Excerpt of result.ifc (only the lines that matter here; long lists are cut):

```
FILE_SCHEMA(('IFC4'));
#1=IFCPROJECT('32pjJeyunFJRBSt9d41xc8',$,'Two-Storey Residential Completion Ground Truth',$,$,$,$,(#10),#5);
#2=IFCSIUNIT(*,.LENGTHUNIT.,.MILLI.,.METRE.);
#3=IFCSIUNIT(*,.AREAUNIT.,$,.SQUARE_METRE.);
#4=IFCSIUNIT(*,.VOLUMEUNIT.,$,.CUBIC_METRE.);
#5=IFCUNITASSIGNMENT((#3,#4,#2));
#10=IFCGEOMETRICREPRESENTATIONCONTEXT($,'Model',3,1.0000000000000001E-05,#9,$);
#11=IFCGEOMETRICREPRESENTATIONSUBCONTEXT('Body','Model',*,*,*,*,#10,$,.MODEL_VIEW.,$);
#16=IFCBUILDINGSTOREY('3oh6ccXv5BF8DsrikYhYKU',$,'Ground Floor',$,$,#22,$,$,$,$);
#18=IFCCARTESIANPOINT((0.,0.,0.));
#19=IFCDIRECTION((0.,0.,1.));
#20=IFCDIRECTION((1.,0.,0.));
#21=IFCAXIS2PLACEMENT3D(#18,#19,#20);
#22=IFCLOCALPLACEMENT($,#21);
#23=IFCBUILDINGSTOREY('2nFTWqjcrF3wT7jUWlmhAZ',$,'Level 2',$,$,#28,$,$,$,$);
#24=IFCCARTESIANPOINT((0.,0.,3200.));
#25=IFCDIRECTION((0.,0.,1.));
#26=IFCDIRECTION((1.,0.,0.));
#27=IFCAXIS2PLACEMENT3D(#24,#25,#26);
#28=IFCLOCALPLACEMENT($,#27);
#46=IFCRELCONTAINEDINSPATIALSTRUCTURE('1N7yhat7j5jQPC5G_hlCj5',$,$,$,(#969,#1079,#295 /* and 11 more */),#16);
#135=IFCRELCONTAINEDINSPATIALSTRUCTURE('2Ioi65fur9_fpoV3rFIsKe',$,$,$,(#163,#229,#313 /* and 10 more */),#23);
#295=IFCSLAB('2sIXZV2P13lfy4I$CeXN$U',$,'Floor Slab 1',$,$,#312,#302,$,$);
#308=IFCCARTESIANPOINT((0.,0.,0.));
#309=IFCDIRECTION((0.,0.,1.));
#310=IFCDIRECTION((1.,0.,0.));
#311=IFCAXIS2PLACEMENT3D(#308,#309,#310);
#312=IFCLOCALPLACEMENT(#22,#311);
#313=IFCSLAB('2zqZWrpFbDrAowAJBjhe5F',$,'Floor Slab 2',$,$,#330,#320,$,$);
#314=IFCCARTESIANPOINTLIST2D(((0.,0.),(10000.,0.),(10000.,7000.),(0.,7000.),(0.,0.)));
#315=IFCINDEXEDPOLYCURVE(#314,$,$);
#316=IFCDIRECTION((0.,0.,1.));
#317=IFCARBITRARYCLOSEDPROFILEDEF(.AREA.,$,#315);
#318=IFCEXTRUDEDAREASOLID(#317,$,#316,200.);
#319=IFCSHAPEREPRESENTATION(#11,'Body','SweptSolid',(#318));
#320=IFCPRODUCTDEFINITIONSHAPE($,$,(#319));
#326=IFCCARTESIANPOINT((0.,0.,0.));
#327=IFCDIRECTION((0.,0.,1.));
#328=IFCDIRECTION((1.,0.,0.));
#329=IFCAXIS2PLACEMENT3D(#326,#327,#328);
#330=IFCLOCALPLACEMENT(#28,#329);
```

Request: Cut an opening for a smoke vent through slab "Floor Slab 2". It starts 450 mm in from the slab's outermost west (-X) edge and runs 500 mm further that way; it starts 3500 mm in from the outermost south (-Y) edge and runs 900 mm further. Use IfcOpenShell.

```python
import numpy as np
import ifcopenshell
import ifcopenshell.api.feature
import ifcopenshell.api.geometry
import ifcopenshell.api.root
import ifcopenshell.geom
import ifcopenshell.util.placement
import ifcopenshell.util.representation
import ifcopenshell.util.shape
import ifcopenshell.util.unit

model = ifcopenshell.open("result.ifc")
unit_scale = ifcopenshell.util.unit.calculate_unit_scale(model)
settings = ifcopenshell.geom.settings()


def volume(element):
    """Net volume in cubic metres, openings subtracted."""
    shape = ifcopenshell.geom.create_shape(settings, element)
    return ifcopenshell.util.shape.get_volume(shape.geometry)


slab = model.by_guid("2zqZWrpFbDrAowAJBjhe5F")
before = volume(slab)

# Extent in the slab's own axes, in metres. The edges named are its -X and -Y sides.
slab_shape = ifcopenshell.geom.create_shape(settings, slab)
vertices = ifcopenshell.util.shape.get_vertices(slab_shape.geometry)
x_min, y_min, bottom = vertices.min(axis=0)
top = vertices[:, 2].max()

opening = ifcopenshell.api.root.create_entity(model, ifc_class="IfcOpeningElement", name="Smoke vent opening", predefined_type="OPENING")
context = ifcopenshell.util.representation.get_context(model, "Model", "Body", "MODEL_VIEW")
width, depth = 0.5, 0.9
outline = [(0.0, 0.0), (width, 0.0), (width, depth), (0.0, depth), (0.0, 0.0)]
# Overshoot both faces by 50 mm so the cut is clean.
shape = ifcopenshell.api.geometry.add_slab_representation(
    model, context=context, depth=top - bottom + 0.1, polyline=outline
)
ifcopenshell.api.geometry.assign_representation(model, product=opening, representation=shape)

matrix = ifcopenshell.util.placement.get_local_placement(slab.ObjectPlacement)
matrix[:, 3] = matrix @ np.append(np.array([x_min + 0.45, y_min + 3.5, bottom - 0.05]) / unit_scale, 1.0)
ifcopenshell.api.geometry.edit_object_placement(model, product=opening, matrix=matrix, is_si=False)
ifcopenshell.api.feature.add_feature(model, feature=opening, element=slab)

after = volume(slab)

print(f"slab volume {before:.3f} -> {after:.3f} m3")

model.write("result-out.ifc")
```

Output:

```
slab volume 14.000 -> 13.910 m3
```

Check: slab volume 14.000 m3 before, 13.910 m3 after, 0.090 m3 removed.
